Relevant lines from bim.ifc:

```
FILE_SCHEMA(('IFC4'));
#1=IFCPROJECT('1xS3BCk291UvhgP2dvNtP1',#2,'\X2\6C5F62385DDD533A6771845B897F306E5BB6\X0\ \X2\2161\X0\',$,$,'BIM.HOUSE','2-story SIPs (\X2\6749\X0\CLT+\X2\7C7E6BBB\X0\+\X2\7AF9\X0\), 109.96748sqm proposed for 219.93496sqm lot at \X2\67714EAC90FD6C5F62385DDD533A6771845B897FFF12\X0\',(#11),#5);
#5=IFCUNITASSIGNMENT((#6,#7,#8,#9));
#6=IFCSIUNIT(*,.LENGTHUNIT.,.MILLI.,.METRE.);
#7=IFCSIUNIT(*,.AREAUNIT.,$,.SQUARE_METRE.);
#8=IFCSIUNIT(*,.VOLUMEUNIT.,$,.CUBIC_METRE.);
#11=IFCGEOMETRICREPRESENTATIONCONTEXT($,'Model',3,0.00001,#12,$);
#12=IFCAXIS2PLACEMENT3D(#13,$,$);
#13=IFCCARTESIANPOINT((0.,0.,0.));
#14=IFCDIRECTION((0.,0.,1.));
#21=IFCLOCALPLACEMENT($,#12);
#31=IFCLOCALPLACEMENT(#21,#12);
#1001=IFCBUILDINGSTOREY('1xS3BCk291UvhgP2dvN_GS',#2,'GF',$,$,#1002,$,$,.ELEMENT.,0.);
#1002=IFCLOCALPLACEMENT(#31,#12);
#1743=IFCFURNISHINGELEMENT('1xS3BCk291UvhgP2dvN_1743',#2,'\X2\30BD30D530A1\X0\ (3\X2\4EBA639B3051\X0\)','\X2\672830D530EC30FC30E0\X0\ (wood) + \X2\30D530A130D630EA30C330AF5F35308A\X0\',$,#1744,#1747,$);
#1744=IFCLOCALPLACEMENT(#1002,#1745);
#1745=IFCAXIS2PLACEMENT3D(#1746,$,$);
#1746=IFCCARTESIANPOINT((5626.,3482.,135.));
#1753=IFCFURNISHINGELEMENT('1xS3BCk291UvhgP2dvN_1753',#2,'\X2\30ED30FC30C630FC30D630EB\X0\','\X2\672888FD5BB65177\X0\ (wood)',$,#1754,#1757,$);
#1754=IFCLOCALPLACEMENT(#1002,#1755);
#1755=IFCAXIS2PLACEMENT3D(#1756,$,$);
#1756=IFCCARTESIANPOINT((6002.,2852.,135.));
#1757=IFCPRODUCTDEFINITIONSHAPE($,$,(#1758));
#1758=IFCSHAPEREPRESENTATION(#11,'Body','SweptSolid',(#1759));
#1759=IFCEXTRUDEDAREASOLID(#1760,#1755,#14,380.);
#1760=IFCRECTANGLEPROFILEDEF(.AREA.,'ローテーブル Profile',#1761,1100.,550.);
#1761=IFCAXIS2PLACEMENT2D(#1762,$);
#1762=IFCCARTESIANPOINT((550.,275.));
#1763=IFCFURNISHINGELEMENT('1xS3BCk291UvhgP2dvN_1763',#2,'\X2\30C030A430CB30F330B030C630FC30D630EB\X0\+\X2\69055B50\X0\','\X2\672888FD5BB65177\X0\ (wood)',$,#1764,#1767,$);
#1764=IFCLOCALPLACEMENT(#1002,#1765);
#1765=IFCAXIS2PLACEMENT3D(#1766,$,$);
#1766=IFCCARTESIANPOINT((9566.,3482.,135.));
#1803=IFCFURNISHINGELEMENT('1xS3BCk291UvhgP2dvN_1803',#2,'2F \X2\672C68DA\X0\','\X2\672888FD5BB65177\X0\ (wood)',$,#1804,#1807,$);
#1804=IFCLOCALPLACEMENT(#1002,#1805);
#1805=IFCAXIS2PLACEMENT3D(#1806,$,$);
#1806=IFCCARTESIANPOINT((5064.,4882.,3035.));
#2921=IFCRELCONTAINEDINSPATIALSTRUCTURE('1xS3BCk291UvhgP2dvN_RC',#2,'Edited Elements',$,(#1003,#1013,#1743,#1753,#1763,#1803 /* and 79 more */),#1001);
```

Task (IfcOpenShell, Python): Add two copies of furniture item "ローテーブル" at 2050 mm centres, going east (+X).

```python
import numpy as np
import ifcopenshell
import ifcopenshell.api.geometry
import ifcopenshell.api.root
import ifcopenshell.util.element
import ifcopenshell.util.placement
import ifcopenshell.util.unit

model = ifcopenshell.open("bim.ifc")
unit_scale = ifcopenshell.util.unit.calculate_unit_scale(model)


def reuse_history(source, copy):
    """copy_class also copies each property set's owner history, people and application; keep the originals."""
    for rel in copy.IsDefinedBy:
        if rel.is_a("IfcRelDefinesByProperties") and (history := rel.RelatingPropertyDefinition.OwnerHistory):
            rel.RelatingPropertyDefinition.OwnerHistory = source.OwnerHistory
            ifcopenshell.util.element.remove_deep2(model, history)


source = model.by_id(1753)
base = ifcopenshell.util.placement.get_local_placement(source.ObjectPlacement)
step = np.array([1.0, 0.0, 0.0]) * 2.05 / unit_scale

for i in range(1, 3):
    copy = ifcopenshell.api.root.copy_class(model, product=source)
    copy.Representation = ifcopenshell.util.element.copy_deep(
        model, source.Representation, exclude=["IfcGeometricRepresentationContext", "IfcRepresentationMap"]
    )
    reuse_history(source, copy)
    matrix = base.copy()
    matrix[:3, 3] += i * step
    print("added at", matrix[:3, 3].round(3) + 0.0)
    ifcopenshell.api.geometry.edit_object_placement(model, product=copy, matrix=matrix, is_si=False)

model.write("bim_updated.ifc")
```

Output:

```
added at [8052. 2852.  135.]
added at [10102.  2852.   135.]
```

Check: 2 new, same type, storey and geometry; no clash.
